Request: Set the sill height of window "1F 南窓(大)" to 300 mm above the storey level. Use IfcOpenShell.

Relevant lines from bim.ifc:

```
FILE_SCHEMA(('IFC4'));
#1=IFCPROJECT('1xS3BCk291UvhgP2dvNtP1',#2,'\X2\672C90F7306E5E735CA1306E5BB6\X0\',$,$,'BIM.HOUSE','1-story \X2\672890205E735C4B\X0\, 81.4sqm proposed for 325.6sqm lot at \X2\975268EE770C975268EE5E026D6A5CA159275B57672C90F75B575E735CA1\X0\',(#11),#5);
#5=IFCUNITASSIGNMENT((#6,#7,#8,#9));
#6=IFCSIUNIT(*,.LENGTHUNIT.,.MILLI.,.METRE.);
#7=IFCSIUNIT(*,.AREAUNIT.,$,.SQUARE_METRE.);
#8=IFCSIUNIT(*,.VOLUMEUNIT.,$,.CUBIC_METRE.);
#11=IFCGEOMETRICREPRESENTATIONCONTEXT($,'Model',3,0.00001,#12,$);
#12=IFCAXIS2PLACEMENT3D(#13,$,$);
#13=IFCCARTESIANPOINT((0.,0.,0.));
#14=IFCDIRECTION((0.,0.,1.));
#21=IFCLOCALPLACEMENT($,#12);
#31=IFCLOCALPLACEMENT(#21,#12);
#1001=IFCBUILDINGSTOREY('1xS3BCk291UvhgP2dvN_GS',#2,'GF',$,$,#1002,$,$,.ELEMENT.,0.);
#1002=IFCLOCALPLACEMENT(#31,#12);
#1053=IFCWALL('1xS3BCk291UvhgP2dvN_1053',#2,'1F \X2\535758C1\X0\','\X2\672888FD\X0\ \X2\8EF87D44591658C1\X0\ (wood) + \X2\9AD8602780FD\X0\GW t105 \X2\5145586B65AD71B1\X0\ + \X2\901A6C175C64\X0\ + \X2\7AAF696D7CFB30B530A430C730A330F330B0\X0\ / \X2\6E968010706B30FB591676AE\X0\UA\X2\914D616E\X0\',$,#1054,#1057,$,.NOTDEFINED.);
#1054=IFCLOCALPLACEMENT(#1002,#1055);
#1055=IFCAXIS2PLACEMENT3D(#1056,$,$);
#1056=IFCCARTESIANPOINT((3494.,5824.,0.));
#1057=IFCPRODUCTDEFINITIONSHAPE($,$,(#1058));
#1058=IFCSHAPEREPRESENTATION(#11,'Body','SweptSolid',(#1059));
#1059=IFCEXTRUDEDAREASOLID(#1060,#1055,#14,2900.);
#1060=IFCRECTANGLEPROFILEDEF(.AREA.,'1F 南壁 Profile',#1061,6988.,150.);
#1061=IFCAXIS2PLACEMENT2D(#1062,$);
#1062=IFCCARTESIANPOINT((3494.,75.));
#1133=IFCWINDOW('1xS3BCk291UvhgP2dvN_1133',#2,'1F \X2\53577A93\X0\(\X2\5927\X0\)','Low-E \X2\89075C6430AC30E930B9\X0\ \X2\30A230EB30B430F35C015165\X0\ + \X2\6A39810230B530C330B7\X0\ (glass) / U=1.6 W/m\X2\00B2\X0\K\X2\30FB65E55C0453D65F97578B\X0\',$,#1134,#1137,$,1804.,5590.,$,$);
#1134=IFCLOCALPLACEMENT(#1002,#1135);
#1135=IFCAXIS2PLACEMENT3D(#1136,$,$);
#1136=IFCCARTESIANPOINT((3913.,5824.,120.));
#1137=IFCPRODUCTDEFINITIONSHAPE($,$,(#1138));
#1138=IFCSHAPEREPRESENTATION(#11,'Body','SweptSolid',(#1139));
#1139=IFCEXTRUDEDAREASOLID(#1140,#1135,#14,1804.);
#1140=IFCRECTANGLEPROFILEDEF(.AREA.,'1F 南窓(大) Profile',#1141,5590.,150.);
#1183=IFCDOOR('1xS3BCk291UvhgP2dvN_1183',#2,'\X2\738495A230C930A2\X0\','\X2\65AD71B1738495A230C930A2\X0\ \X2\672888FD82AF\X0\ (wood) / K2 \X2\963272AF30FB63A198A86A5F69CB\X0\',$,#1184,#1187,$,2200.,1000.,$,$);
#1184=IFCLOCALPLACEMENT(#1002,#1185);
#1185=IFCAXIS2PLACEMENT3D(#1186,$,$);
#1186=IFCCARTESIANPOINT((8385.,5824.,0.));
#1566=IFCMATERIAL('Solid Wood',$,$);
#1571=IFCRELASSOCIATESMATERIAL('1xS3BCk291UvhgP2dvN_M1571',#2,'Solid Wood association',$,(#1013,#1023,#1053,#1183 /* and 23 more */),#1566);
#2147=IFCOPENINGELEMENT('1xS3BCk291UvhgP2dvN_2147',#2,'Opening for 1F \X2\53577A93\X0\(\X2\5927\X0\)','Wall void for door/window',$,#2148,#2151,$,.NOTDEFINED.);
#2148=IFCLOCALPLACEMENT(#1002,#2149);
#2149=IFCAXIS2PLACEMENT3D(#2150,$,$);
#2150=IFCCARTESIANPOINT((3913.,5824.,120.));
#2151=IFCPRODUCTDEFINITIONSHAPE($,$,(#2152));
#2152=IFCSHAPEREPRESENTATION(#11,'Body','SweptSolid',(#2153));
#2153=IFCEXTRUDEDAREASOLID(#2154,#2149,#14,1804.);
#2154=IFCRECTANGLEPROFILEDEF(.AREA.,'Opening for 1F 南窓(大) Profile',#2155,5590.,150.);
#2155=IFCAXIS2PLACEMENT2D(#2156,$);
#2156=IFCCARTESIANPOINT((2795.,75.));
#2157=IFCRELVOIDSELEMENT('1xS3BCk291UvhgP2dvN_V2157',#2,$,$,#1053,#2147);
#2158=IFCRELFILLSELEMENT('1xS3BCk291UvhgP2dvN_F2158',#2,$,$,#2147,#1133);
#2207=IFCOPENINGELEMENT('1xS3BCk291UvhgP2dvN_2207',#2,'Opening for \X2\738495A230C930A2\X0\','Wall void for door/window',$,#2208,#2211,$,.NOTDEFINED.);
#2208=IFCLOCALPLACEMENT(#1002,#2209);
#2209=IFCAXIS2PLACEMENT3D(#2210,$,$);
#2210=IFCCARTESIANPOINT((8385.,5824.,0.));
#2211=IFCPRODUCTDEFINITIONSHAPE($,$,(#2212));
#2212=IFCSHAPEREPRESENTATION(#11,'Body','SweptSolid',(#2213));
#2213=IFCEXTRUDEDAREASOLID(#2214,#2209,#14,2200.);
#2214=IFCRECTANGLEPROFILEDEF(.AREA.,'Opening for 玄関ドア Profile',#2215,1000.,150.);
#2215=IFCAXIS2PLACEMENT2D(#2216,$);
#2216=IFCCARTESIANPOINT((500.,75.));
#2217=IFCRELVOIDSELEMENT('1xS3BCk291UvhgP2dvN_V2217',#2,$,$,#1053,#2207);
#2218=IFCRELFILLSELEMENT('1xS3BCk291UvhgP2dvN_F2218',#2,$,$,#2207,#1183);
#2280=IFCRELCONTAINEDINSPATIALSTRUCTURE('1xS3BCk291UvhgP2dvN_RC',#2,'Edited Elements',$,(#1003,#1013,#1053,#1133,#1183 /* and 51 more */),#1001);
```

```python
import numpy as np
import ifcopenshell
import ifcopenshell.api.geometry
import ifcopenshell.geom
import ifcopenshell.util.element
import ifcopenshell.util.placement
import ifcopenshell.util.shape
import ifcopenshell.util.unit

model = ifcopenshell.open("bim.ifc")
unit_scale = ifcopenshell.util.unit.calculate_unit_scale(model)

window = model.by_guid("1xS3BCk291UvhgP2dvN_1133")
opening = window.FillsVoids[0].RelatingOpeningElement
storey = ifcopenshell.util.element.get_container(window, ifc_class="IfcBuildingStorey")
level = ifcopenshell.util.placement.get_local_placement(storey.ObjectPlacement)[2, 3]

# The opening's origin need not be at the sill, so measure its lowest point.
shape = ifcopenshell.geom.create_shape(ifcopenshell.geom.settings(), opening)
bottom = ifcopenshell.util.shape.get_shape_bottom_elevation(shape, shape.geometry) / unit_scale
dz = level + 300.0 - bottom

shift = np.array([0.0, 0.0, dz])
# The window is not placed relative to its opening, so move both.
for product in (opening, window):
    matrix = ifcopenshell.util.placement.get_local_placement(product.ObjectPlacement)
    matrix[:3, 3] += shift
    ifcopenshell.api.geometry.edit_object_placement(model, product=product, matrix=matrix, is_si=False)

print(f"moved by {dz * unit_scale:+.3f} m")

model.write("bim_edited.ifc")
```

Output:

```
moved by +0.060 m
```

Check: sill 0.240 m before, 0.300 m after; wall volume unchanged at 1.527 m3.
